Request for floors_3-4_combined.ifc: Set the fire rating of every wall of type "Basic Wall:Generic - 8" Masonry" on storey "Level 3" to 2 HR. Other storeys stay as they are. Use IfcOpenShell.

First a look at what the model holds.

```python
import ifcopenshell
import ifcopenshell.util.element

model = ifcopenshell.open("floors_3-4_combined.ifc")
print(model.schema)
storey = next(s for s in model.by_type("IfcBuildingStorey") if s.Name == "Level 3")
walls = [e for e in ifcopenshell.util.element.get_decomposition(storey) if e.is_a("IfcWall")]
seen = {}
for e in walls:
    element_type = ifcopenshell.util.element.get_type(e)
    key = (element_type.Name if element_type != e and element_type else None, ifcopenshell.util.element.get_pset(e, "Pset_WallCommon", "FireRating"))
    seen[key] = seen.get(key, 0) + 1
for (name, value), count in sorted(seen.items(), key=str):
    print(count, "x", name, "|", value)
```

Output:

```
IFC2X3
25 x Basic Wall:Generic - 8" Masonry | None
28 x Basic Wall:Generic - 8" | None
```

```python
import ifcopenshell
import ifcopenshell.api.pset
import ifcopenshell.util.element

model = ifcopenshell.open("floors_3-4_combined.ifc")

storey = next(s for s in model.by_type("IfcBuildingStorey") if s.Name == "Level 3")
walls = [e for e in ifcopenshell.util.element.get_decomposition(storey) if e.is_a("IfcWall")]

count = 0
for e in walls:
    element_type = ifcopenshell.util.element.get_type(e)
    if element_type in (None, e) or element_type.Name != 'Basic Wall:Generic - 8" Masonry':
        continue
    # add_pset returns the element's existing set when there is one.
    pset = ifcopenshell.api.pset.add_pset(model, product=e, name="Pset_WallCommon")
    ifcopenshell.api.pset.edit_pset(model, pset=pset, properties={"FireRating": "2 HR"})
    count += 1

print(count, "walls updated")

model.write("floors_3-4_combined_updated.ifc")
```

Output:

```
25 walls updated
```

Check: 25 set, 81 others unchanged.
